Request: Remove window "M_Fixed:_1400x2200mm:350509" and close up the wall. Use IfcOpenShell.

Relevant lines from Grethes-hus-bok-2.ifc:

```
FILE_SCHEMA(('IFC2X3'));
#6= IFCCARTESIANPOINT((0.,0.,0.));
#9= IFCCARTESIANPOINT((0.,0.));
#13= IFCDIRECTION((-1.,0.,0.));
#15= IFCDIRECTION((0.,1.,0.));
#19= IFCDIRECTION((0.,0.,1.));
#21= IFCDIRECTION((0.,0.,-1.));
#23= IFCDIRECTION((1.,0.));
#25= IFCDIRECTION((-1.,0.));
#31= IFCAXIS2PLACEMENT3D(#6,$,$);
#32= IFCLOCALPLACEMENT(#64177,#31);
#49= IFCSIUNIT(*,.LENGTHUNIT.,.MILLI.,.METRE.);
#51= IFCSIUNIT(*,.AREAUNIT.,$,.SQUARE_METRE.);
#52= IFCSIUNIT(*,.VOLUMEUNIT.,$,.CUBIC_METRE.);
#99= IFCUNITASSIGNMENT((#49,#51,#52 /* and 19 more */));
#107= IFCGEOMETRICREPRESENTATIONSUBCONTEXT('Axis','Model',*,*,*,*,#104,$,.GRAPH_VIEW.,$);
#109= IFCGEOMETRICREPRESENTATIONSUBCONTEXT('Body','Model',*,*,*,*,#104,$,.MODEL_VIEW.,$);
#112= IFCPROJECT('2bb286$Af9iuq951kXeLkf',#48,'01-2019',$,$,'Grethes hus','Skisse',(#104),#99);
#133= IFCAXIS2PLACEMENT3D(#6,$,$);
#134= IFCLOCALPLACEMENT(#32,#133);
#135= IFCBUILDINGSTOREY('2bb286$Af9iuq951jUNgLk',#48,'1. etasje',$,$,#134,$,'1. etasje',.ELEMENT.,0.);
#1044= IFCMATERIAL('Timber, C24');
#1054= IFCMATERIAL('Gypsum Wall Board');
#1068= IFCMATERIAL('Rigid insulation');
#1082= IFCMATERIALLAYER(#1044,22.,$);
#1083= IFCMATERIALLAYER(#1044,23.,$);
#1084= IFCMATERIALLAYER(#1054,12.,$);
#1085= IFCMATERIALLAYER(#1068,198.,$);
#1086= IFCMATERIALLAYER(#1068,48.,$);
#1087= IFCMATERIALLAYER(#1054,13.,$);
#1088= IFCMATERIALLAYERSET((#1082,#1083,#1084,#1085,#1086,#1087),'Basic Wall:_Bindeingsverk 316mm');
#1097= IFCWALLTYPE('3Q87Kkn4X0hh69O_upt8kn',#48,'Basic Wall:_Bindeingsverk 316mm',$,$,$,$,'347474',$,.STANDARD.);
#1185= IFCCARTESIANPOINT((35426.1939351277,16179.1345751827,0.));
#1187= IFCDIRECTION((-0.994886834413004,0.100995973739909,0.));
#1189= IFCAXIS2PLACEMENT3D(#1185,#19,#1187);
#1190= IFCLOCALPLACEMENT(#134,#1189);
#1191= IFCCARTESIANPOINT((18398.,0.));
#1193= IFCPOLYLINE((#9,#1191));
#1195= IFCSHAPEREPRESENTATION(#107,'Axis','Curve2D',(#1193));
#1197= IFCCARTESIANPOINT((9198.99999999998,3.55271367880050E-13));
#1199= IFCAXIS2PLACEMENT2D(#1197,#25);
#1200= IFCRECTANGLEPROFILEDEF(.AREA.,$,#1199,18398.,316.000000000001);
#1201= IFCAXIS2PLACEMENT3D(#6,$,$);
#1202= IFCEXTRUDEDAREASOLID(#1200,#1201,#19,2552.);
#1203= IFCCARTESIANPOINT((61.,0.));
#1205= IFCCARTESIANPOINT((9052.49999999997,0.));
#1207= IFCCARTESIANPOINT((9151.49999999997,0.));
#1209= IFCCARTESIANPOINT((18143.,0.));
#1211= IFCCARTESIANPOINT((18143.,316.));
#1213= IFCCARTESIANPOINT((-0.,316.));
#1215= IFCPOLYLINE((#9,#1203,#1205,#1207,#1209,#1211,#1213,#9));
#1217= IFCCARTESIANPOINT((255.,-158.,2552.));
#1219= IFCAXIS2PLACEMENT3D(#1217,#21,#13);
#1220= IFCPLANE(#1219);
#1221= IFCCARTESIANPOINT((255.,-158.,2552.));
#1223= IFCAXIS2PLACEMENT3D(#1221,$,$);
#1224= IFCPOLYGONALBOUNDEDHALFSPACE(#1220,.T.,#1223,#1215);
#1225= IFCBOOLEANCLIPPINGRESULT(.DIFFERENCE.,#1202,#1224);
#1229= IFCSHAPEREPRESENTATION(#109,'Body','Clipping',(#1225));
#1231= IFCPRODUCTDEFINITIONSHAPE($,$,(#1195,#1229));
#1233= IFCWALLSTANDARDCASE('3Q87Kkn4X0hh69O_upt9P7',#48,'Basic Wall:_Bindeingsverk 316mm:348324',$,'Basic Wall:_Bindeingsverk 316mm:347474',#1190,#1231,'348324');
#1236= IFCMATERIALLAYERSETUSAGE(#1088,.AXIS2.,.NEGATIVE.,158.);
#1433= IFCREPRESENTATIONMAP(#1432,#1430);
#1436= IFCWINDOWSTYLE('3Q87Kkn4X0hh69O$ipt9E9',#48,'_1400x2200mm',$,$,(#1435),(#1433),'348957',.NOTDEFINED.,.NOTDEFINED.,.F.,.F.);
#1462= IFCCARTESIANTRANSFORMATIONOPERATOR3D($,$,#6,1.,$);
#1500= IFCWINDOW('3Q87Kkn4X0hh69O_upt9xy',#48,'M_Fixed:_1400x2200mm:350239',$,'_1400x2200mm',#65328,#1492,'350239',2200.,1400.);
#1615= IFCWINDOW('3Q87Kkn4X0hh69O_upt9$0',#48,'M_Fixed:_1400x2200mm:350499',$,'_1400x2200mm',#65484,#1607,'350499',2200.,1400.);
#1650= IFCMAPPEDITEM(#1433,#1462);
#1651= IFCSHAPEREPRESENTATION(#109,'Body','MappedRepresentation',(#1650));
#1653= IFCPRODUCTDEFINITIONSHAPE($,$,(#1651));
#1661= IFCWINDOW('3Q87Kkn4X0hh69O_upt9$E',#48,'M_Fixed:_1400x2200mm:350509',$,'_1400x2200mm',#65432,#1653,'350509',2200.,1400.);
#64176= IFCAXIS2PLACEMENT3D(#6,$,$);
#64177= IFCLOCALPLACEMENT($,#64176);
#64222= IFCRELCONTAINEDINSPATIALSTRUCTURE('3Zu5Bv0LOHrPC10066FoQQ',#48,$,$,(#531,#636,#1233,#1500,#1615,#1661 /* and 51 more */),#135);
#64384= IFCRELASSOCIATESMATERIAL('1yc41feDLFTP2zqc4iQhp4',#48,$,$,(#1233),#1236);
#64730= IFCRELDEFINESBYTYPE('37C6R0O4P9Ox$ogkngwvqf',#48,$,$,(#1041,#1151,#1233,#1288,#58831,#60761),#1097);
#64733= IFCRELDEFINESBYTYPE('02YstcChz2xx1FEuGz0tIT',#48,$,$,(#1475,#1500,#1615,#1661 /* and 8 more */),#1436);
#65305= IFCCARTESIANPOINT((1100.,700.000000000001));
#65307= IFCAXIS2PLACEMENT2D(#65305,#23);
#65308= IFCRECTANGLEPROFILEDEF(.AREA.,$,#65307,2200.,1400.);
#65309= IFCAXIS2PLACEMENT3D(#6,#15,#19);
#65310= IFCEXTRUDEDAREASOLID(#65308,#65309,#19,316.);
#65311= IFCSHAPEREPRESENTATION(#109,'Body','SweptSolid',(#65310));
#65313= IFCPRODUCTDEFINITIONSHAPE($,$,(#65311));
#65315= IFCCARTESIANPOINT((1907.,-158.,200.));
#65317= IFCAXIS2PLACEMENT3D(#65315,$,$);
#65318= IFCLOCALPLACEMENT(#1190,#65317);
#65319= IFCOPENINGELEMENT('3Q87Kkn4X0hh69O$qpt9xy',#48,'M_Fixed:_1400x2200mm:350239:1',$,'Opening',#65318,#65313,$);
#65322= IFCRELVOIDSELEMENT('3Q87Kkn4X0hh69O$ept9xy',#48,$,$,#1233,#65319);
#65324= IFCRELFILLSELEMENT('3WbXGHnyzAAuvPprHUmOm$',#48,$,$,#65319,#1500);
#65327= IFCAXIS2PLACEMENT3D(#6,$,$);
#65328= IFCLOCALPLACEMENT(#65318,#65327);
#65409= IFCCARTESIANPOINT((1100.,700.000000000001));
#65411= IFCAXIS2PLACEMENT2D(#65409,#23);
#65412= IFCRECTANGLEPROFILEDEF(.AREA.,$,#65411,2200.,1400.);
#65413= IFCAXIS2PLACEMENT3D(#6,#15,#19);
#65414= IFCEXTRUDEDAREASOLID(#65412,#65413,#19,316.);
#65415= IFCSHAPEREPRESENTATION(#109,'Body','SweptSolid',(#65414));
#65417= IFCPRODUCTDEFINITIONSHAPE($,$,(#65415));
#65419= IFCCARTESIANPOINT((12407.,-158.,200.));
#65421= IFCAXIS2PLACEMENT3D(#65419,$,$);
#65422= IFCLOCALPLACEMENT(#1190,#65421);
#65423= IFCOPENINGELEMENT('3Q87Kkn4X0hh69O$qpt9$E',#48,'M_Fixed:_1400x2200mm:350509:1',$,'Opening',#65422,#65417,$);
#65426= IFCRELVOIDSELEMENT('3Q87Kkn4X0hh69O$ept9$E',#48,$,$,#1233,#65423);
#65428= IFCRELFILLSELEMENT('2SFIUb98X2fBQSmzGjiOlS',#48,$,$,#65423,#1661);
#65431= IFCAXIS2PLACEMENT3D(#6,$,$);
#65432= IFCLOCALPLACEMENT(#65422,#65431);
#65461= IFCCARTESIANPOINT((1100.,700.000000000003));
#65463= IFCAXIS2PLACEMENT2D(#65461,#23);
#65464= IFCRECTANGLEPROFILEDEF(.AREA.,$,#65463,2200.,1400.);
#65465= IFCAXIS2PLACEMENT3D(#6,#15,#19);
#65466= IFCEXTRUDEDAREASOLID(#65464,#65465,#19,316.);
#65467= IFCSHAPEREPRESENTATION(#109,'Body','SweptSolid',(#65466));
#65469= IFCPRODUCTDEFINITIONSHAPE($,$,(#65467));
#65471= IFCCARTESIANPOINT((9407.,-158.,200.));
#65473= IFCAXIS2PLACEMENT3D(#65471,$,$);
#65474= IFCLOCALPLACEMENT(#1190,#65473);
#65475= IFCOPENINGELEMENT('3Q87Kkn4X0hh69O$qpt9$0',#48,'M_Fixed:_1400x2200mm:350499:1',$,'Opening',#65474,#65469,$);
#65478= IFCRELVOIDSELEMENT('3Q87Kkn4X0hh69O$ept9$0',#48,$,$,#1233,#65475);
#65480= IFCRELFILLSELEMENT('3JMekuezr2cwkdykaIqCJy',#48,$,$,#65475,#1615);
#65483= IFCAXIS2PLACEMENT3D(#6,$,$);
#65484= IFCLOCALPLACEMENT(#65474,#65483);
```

```python
import ifcopenshell
import ifcopenshell.api.feature
import ifcopenshell.api.root
import ifcopenshell.geom
import ifcopenshell.util.shape

model = ifcopenshell.open("Grethes-hus-bok-2.ifc")
settings = ifcopenshell.geom.settings()


def volume(element):
    """Net volume in cubic metres, openings subtracted."""
    shape = ifcopenshell.geom.create_shape(settings, element)
    return ifcopenshell.util.shape.get_volume(shape.geometry)


window = model.by_id(1661)
opening = window.FillsVoids[0].RelatingOpeningElement
wall = opening.VoidsElements[0].RelatingBuildingElement
before = volume(wall)

ifcopenshell.api.root.remove_product(model, product=window)
ifcopenshell.api.feature.remove_feature(model, feature=opening)

after = volume(wall)

print(f"wall volume {before:.3f} -> {after:.3f} m3")

model.write("Grethes-hus-bok-2_updated.ifc")
```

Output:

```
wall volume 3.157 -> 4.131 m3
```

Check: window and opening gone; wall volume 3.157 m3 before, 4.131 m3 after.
